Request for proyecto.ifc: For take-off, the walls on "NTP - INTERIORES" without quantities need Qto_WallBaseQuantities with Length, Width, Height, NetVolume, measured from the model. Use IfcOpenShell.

First a look at what the model holds.

```python
import ifcopenshell
import ifcopenshell.util.element
import ifcopenshell.util.unit

model = ifcopenshell.open("proyecto.ifc")
print(model.schema)
for unit_type in ("LENGTHUNIT", "AREAUNIT", "VOLUMEUNIT"):
    print(unit_type, ifcopenshell.util.unit.calculate_unit_scale(model, unit_type))
storey = next(s for s in model.by_type("IfcBuildingStorey") if s.Name == "NTP - INTERIORES")
walls = [e for e in ifcopenshell.util.element.get_decomposition(storey) if e.is_a("IfcWall")]
for e in sorted(walls, key=lambda e: e.id()):
    print(e.id(), e.is_a(), e.Name, list(ifcopenshell.util.element.get_psets(e, qtos_only=True)), sep=" | ")
```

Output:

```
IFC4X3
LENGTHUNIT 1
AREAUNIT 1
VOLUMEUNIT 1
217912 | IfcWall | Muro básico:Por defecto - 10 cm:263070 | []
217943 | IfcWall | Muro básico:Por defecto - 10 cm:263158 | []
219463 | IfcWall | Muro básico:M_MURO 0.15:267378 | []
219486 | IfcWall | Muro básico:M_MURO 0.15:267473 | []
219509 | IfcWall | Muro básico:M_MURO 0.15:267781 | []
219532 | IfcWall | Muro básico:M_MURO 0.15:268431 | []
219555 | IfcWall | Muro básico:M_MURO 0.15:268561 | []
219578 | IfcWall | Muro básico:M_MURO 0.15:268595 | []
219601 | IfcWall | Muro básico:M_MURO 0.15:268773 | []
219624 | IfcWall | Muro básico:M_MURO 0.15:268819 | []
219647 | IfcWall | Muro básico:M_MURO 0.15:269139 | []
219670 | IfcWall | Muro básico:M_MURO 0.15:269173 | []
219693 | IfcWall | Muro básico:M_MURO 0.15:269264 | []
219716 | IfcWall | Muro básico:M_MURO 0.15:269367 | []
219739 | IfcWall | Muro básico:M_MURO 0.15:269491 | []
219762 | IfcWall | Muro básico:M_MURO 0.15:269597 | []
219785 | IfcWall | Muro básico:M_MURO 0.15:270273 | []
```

```python
import ifcopenshell
import ifcopenshell.api.pset
import ifcopenshell.geom
import ifcopenshell.util.element
import ifcopenshell.util.shape
import ifcopenshell.util.unit

model = ifcopenshell.open("proyecto.ifc")
unit_scale = ifcopenshell.util.unit.calculate_unit_scale(model)
volume_scale = ifcopenshell.util.unit.calculate_unit_scale(model, "VOLUMEUNIT")
settings = ifcopenshell.geom.settings()

storey = next(s for s in model.by_type("IfcBuildingStorey") if s.Name == "NTP - INTERIORES")
walls = [e for e in ifcopenshell.util.element.get_decomposition(storey) if e.is_a("IfcWall")]

for e in sorted(walls, key=lambda e: e.id()):
    if ifcopenshell.util.element.get_psets(e, qtos_only=True, should_inherit=False):
        continue
    # Geometry comes back in metres, in the element's own axes.
    shape = ifcopenshell.geom.create_shape(settings, e)
    values = {
        "Length": ifcopenshell.util.shape.get_x(shape.geometry) / unit_scale,
        "Width": ifcopenshell.util.shape.get_y(shape.geometry) / unit_scale,
        "Height": ifcopenshell.util.shape.get_z(shape.geometry) / unit_scale,
        "NetVolume": ifcopenshell.util.shape.get_volume(shape.geometry) / volume_scale,
    }
    qto = ifcopenshell.api.pset.add_qto(model, product=e, name="Qto_WallBaseQuantities")
    ifcopenshell.api.pset.edit_qto(model, qto=qto, properties=values)
    print(e.id(), {k: round(v, 3) for k, v in values.items()})

model.write("proyecto_edited.ifc")
```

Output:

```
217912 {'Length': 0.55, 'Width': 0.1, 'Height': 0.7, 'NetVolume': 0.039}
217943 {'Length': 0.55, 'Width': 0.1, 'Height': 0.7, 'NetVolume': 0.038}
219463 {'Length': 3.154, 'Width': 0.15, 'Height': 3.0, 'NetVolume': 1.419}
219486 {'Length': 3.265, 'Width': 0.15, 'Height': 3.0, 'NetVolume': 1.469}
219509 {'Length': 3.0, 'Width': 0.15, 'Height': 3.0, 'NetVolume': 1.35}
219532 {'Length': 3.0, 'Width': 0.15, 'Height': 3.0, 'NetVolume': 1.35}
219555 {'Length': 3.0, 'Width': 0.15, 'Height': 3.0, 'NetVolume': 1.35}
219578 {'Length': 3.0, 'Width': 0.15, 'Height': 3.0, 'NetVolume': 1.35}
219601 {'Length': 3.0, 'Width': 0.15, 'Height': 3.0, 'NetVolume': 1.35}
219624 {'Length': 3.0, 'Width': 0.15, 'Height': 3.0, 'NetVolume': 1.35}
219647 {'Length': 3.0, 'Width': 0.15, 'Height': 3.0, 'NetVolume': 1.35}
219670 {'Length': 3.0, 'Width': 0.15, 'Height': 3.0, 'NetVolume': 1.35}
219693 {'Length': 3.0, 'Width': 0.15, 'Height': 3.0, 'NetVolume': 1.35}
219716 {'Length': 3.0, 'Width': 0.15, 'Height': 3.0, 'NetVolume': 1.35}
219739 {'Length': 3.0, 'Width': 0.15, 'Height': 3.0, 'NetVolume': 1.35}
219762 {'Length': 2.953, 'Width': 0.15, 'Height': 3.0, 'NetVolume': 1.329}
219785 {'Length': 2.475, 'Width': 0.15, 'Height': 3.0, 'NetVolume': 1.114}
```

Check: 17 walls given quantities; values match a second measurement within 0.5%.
